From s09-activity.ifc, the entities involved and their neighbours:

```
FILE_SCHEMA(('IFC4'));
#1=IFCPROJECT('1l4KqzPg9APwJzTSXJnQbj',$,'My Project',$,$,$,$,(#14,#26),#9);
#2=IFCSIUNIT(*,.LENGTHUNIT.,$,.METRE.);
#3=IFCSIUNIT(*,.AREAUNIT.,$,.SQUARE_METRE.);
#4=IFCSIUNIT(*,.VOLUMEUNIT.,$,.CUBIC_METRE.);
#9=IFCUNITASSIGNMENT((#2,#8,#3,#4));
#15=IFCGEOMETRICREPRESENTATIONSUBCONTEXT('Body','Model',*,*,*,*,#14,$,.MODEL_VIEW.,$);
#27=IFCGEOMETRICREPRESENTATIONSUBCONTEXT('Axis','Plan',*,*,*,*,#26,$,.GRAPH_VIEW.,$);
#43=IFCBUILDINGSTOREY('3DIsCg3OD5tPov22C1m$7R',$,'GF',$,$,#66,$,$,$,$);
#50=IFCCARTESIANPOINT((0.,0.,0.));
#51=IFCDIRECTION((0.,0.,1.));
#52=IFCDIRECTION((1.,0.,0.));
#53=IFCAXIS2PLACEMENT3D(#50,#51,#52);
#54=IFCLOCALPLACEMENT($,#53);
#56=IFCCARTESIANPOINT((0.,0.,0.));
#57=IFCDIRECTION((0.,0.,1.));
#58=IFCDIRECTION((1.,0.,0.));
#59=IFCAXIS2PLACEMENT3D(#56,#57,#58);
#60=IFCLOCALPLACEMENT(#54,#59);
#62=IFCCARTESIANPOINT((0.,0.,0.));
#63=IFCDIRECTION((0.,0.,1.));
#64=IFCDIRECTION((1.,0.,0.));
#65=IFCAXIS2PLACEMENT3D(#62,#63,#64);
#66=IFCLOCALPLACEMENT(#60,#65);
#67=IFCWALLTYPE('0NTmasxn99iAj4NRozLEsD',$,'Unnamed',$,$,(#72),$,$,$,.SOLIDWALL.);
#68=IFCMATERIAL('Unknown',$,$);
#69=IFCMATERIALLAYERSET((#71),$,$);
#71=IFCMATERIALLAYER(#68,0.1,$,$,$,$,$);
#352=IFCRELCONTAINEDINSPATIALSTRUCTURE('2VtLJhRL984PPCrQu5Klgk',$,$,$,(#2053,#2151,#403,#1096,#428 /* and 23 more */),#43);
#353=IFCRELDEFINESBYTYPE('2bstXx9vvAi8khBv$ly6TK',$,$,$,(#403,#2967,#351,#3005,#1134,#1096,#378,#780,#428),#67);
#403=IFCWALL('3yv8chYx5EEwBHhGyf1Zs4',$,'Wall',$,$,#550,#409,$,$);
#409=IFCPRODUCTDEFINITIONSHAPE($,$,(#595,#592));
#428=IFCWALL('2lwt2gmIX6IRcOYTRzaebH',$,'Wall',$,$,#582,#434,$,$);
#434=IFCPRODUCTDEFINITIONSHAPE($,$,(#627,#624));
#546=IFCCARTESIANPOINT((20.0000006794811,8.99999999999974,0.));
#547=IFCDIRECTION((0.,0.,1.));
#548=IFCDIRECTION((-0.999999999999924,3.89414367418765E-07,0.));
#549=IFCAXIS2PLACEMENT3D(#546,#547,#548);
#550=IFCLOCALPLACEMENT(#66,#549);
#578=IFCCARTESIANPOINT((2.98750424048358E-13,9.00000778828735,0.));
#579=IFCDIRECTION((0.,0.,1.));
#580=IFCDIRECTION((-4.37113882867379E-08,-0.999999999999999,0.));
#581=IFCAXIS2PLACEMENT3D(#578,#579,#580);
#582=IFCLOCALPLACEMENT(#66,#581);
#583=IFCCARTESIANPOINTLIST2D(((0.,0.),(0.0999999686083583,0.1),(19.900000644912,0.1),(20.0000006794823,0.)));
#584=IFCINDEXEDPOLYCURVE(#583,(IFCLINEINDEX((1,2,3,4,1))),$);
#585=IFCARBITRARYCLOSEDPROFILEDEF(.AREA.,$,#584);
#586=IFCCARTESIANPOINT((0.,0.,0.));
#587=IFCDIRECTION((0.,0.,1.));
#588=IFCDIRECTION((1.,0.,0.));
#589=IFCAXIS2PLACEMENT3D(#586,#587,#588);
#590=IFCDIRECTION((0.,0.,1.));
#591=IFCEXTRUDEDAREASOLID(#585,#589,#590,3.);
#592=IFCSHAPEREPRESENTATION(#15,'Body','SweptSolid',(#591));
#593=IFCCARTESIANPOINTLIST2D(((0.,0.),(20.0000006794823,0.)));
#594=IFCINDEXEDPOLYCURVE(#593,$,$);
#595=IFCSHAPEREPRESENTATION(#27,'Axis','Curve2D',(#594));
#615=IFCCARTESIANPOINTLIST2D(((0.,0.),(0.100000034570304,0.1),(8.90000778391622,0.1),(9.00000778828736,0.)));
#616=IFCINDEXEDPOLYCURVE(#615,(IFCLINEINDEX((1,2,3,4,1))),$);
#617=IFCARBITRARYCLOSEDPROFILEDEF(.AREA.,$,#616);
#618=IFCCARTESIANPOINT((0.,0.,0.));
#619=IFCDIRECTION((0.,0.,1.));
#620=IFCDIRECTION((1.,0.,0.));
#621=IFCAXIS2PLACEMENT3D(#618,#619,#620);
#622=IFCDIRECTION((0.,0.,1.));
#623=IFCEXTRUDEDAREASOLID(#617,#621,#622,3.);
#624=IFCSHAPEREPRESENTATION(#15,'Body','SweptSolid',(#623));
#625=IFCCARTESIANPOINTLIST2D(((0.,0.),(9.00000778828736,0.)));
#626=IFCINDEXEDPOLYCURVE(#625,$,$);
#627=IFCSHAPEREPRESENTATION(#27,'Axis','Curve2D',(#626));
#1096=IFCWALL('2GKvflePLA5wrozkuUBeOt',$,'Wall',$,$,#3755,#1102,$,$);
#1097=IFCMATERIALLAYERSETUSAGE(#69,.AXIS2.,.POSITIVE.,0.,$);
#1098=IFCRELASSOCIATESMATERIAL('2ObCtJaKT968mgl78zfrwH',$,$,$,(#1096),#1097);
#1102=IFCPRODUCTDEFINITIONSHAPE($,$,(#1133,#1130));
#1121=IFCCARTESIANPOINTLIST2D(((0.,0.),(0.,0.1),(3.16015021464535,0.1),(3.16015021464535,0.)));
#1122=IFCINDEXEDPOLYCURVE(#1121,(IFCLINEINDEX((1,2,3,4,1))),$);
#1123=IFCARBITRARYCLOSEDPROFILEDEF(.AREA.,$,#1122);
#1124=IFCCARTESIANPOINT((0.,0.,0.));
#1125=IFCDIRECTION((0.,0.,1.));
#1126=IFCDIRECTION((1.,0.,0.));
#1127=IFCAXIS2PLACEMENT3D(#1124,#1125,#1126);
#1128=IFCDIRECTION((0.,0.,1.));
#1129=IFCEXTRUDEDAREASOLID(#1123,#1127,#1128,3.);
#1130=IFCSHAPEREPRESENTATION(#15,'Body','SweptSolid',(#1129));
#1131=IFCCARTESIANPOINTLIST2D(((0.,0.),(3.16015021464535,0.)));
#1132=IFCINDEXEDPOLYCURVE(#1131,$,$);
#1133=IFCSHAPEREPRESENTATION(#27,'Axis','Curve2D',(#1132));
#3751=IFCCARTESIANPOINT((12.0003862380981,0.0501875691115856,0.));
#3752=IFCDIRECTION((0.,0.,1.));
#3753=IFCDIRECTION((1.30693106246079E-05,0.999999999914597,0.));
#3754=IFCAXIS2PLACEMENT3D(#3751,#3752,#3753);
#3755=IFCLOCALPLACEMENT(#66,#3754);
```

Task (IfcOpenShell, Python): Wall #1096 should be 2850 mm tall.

```python
import ifcopenshell
import ifcopenshell.geom
import ifcopenshell.util.representation
import ifcopenshell.util.shape
import ifcopenshell.util.unit

model = ifcopenshell.open("s09-activity.ifc")
unit_scale = ifcopenshell.util.unit.calculate_unit_scale(model)
settings = ifcopenshell.geom.settings()


def volume(element):
    """Net volume in cubic metres, openings subtracted."""
    shape = ifcopenshell.geom.create_shape(settings, element)
    return ifcopenshell.util.shape.get_volume(shape.geometry)


wall = model.by_guid("2GKvflePLA5wrozkuUBeOt")
before = volume(wall)

body = ifcopenshell.util.representation.get_representation(wall, "Model", "Body")
solid = body.Items[0]
old_height = solid.Depth
solid.Depth = 2.85 / unit_scale
after = volume(wall)

print(f"height {old_height:g} -> {solid.Depth:g}, volume {before:.3f} -> {after:.3f} m3")

model.write("s09-activity-out.ifc")
```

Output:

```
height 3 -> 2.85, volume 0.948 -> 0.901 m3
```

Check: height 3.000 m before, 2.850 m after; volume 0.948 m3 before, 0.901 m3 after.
